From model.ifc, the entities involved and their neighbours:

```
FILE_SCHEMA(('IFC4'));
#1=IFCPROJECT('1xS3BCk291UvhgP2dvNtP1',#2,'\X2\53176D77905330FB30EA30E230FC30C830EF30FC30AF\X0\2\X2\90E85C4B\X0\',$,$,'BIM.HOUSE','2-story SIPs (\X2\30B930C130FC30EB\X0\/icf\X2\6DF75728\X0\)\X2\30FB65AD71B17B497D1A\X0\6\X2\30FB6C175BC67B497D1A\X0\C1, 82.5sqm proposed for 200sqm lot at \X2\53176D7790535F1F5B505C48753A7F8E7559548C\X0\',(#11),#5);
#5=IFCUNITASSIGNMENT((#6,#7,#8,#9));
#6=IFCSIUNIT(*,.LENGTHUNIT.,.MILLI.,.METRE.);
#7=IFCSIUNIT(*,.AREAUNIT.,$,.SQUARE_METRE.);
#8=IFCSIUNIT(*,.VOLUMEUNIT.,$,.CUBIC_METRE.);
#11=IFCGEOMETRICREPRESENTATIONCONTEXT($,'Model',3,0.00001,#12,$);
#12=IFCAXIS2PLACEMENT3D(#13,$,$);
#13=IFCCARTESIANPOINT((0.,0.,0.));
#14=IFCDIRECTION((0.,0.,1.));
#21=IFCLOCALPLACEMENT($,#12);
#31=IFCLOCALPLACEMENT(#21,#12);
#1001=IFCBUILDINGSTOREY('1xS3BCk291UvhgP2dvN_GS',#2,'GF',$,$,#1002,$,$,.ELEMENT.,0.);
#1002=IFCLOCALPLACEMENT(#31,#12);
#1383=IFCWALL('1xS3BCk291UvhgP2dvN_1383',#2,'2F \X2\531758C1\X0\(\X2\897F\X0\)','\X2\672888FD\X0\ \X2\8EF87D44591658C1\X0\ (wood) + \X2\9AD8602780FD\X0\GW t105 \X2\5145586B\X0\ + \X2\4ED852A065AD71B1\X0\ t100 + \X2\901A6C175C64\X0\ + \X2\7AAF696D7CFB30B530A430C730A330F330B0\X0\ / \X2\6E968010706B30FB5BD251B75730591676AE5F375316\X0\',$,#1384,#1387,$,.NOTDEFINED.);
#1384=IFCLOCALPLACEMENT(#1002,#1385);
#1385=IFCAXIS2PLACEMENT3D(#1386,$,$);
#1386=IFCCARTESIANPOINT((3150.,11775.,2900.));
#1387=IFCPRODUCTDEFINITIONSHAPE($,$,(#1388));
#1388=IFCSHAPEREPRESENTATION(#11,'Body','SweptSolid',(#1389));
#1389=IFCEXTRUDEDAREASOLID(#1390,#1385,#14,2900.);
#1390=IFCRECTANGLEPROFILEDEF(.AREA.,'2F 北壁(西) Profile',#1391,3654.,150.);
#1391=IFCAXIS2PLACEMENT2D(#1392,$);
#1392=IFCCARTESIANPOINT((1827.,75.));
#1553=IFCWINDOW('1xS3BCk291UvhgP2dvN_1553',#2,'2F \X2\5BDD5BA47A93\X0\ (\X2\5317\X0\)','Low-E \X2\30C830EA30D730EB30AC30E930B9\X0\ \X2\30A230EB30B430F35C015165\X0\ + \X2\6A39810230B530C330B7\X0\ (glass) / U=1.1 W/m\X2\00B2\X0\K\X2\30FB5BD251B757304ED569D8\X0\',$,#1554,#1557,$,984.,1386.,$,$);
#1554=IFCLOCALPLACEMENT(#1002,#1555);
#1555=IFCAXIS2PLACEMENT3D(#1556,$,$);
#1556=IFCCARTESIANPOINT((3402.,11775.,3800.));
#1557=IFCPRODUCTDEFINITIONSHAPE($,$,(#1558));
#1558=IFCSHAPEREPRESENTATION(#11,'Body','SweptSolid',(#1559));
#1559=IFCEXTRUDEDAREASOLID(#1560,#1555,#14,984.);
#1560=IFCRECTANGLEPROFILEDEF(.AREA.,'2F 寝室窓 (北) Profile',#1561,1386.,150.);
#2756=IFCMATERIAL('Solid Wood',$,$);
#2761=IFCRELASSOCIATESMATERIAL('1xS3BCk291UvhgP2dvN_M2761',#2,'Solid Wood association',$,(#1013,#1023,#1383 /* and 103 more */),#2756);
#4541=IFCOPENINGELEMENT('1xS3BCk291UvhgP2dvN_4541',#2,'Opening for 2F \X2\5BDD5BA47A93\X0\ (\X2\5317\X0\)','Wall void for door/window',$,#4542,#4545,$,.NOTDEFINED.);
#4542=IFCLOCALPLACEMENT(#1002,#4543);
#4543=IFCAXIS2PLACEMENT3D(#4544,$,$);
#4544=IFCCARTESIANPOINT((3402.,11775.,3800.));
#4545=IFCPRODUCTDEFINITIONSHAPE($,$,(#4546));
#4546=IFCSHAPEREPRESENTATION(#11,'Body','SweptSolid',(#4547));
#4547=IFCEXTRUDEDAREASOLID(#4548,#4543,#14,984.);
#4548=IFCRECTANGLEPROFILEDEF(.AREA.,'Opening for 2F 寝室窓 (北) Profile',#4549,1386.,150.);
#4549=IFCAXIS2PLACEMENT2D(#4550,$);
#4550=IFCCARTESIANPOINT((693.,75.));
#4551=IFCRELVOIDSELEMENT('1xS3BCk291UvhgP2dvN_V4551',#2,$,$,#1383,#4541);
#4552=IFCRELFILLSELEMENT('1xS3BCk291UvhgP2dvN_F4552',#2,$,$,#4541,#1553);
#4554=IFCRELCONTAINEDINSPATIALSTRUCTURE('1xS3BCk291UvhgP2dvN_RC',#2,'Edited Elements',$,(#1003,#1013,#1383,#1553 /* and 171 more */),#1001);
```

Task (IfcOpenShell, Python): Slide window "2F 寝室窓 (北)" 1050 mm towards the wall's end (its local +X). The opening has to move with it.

```python
import ifcopenshell
import ifcopenshell.api.geometry
import ifcopenshell.util.placement

model = ifcopenshell.open("model.ifc")

window = model.by_guid("1xS3BCk291UvhgP2dvN_1553")
opening = window.FillsVoids[0].RelatingOpeningElement
wall = opening.VoidsElements[0].RelatingBuildingElement

wall_matrix = ifcopenshell.util.placement.get_local_placement(wall.ObjectPlacement)
shift = wall_matrix[:3, 0] * 1050.0
before = ifcopenshell.util.placement.get_local_placement(window.ObjectPlacement)[:3, 3].copy()

# The window is not placed relative to its opening, so move both.
for product in (opening, window):
    matrix = ifcopenshell.util.placement.get_local_placement(product.ObjectPlacement)
    matrix[:3, 3] += shift
    ifcopenshell.api.geometry.edit_object_placement(model, product=product, matrix=matrix, is_si=False)

after = ifcopenshell.util.placement.get_local_placement(window.ObjectPlacement)[:3, 3]
print("window moved by", (after - before).round(3) + 0.0)

model.write("model-out.ifc")
```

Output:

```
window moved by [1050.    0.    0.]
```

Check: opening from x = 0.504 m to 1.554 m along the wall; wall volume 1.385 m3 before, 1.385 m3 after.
